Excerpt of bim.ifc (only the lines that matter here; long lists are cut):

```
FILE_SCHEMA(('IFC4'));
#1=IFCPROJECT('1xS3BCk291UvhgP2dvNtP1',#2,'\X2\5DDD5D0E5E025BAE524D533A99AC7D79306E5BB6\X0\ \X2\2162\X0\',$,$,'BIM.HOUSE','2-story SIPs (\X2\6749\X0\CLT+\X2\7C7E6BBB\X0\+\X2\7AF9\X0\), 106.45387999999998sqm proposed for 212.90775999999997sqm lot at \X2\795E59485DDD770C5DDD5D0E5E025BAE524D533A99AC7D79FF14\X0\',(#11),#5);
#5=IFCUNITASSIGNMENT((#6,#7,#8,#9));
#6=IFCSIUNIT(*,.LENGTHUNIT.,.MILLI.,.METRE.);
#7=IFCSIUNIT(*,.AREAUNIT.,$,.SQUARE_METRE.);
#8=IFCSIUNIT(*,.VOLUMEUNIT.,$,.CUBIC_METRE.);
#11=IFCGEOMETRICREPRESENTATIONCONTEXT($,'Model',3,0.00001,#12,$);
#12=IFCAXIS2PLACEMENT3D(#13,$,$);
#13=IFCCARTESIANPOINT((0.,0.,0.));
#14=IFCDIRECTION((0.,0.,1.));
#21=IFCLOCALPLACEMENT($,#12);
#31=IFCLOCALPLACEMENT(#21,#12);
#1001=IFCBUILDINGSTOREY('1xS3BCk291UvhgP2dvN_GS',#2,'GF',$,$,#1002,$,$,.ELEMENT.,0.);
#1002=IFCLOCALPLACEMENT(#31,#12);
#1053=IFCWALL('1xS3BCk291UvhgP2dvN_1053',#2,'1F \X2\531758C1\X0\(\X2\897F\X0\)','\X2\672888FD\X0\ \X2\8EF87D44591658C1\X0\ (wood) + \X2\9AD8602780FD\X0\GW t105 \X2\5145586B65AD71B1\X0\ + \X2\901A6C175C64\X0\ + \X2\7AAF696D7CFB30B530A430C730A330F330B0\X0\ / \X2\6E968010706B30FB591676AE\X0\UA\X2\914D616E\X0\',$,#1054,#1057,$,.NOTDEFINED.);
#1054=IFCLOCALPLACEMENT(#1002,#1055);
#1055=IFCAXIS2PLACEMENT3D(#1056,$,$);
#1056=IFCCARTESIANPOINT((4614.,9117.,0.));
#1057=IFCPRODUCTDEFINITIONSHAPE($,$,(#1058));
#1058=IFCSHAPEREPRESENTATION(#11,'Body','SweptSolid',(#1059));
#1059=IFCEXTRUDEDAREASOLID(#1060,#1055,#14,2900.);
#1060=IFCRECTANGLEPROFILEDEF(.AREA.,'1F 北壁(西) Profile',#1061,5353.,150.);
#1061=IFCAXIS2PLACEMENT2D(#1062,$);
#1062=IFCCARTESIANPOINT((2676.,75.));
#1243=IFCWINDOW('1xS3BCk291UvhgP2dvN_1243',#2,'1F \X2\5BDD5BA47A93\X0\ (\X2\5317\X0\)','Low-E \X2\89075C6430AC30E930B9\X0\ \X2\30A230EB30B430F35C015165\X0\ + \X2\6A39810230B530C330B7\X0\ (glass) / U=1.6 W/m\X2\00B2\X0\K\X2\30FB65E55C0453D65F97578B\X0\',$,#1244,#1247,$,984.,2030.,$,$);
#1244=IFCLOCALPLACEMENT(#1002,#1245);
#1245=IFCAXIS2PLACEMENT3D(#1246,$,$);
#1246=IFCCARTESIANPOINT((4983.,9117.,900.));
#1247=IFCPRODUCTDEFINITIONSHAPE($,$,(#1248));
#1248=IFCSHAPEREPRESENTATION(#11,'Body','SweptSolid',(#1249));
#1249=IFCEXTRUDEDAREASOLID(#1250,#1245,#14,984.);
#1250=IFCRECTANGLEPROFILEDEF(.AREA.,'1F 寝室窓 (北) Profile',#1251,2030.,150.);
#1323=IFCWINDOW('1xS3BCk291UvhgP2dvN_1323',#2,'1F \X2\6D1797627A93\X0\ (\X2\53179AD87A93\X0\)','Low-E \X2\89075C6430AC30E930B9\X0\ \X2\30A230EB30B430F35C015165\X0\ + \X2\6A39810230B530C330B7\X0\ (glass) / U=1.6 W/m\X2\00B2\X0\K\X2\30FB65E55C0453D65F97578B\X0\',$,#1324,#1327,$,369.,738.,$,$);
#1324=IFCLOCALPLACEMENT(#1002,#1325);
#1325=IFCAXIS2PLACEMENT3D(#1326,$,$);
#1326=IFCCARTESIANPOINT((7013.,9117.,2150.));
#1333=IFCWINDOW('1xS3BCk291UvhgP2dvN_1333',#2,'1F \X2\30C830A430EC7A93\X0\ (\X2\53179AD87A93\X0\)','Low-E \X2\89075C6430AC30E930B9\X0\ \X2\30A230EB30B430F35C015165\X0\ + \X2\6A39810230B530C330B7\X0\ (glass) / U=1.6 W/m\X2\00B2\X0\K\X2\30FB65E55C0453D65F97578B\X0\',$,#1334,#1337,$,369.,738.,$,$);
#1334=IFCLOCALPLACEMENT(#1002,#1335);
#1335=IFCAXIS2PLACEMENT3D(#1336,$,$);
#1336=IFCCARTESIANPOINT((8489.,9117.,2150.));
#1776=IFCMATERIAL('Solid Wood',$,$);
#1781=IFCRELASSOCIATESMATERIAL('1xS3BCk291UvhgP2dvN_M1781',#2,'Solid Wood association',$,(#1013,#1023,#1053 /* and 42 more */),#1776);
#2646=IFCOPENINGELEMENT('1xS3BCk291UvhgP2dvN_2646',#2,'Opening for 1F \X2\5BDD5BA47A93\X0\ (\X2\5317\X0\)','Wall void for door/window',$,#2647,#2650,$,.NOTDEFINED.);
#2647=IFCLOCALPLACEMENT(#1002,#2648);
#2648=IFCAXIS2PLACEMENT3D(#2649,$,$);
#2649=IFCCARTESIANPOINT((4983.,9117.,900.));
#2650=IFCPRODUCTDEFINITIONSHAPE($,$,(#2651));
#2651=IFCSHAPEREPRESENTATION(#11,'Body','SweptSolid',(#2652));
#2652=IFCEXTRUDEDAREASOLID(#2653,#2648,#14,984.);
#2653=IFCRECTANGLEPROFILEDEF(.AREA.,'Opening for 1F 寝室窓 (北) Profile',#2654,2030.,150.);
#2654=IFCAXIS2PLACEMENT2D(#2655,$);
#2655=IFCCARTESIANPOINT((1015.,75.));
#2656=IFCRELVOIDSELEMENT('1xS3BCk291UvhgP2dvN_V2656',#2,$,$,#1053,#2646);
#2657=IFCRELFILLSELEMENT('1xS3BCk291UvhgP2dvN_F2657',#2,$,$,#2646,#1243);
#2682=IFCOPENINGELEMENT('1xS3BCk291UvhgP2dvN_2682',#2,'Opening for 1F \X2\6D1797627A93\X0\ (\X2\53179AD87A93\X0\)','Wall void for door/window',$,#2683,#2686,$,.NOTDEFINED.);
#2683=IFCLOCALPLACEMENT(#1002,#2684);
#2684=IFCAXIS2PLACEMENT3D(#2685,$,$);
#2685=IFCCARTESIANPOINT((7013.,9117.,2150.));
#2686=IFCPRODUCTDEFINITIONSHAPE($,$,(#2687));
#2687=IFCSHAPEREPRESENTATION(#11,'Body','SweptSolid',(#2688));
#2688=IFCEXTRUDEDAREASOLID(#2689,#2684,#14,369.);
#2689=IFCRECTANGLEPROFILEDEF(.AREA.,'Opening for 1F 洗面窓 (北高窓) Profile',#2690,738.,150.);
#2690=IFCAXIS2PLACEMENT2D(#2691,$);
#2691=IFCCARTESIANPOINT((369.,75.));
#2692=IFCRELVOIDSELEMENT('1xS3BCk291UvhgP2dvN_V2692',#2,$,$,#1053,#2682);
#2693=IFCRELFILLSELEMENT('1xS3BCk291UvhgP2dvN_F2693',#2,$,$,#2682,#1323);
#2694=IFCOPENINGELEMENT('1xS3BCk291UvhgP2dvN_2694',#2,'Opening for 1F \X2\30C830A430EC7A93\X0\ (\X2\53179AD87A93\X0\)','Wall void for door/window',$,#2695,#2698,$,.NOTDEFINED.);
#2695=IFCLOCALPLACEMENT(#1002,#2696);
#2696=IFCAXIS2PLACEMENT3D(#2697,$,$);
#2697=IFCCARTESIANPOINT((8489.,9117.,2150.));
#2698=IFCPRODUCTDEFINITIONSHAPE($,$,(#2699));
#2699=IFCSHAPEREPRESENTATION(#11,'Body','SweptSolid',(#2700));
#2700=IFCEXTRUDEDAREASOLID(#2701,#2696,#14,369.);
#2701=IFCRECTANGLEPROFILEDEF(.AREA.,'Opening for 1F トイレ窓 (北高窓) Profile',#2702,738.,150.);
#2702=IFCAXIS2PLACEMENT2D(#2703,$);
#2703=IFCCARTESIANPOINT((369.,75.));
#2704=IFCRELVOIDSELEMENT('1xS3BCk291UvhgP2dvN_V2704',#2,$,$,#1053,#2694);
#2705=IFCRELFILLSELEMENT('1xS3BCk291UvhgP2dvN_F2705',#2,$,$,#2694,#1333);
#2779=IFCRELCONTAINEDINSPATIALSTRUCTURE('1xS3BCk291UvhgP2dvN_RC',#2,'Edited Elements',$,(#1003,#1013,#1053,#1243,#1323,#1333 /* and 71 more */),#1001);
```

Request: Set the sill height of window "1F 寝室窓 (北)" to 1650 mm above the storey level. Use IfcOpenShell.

```python
import numpy as np
import ifcopenshell
import ifcopenshell.api.geometry
import ifcopenshell.geom
import ifcopenshell.util.element
import ifcopenshell.util.placement
import ifcopenshell.util.shape
import ifcopenshell.util.unit

model = ifcopenshell.open("bim.ifc")
unit_scale = ifcopenshell.util.unit.calculate_unit_scale(model)

window = model.by_id(1243)
opening = window.FillsVoids[0].RelatingOpeningElement
storey = ifcopenshell.util.element.get_container(window, ifc_class="IfcBuildingStorey")
level = ifcopenshell.util.placement.get_local_placement(storey.ObjectPlacement)[2, 3]

# The opening's origin need not be at the sill, so measure its lowest point.
shape = ifcopenshell.geom.create_shape(ifcopenshell.geom.settings(), opening)
bottom = ifcopenshell.util.shape.get_shape_bottom_elevation(shape, shape.geometry) / unit_scale
dz = level + 1.65 / unit_scale - bottom

shift = np.array([0.0, 0.0, dz])
# The window is not placed relative to its opening, so move both.
for product in (opening, window):
    matrix = ifcopenshell.util.placement.get_local_placement(product.ObjectPlacement)
    matrix[:3, 3] += shift
    ifcopenshell.api.geometry.edit_object_placement(model, product=product, matrix=matrix, is_si=False)

print(f"moved by {dz * unit_scale:+.3f} m")

model.write("bim_edited.ifc")
```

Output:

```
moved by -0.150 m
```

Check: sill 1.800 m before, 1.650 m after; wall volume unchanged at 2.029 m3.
